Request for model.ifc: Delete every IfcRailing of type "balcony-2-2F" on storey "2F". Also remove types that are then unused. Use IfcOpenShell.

First a look at what the model holds.

```python
import ifcopenshell
import ifcopenshell.util.element

model = ifcopenshell.open("model.ifc")
print(model.schema)
storey = next(s for s in model.by_type("IfcBuildingStorey") if s.Name == "2F")
railings = [e for e in ifcopenshell.util.element.get_decomposition(storey) if e.is_a("IfcRailing")]
seen = {}
for e in railings:
    element_type = ifcopenshell.util.element.get_type(e)
    name = element_type.Name if element_type not in (None, e) else None
    seen[name] = seen.get(name, 0) + 1
for name, count in sorted(seen.items(), key=str):
    print(count, "x", name)
```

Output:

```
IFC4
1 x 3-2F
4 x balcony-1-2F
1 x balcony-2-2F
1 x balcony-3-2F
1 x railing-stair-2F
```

```python
import ifcopenshell
import ifcopenshell.api.root
import ifcopenshell.util.element

model = ifcopenshell.open("model.ifc")

storey = next(s for s in model.by_type("IfcBuildingStorey") if s.Name == "2F")
railings = [e for e in ifcopenshell.util.element.get_decomposition(storey) if e.is_a("IfcRailing")]
targets = [e for e in railings if (t := ifcopenshell.util.element.get_type(e)) not in (None, e) and t.Name == "balcony-2-2F"]
types = {ifcopenshell.util.element.get_type(e) for e in targets} - {None, *targets}

for e in targets:
    ifcopenshell.api.root.remove_product(model, product=e)
print(len(targets), "removed")

unused = [t for t in types if not ifcopenshell.util.element.get_types(t)]
for t in unused:
    ifcopenshell.api.root.remove_product(model, product=t)
print(len(unused), "unused types removed")

model.write("model_v2.ifc")
```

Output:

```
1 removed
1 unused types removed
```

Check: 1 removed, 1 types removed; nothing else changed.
